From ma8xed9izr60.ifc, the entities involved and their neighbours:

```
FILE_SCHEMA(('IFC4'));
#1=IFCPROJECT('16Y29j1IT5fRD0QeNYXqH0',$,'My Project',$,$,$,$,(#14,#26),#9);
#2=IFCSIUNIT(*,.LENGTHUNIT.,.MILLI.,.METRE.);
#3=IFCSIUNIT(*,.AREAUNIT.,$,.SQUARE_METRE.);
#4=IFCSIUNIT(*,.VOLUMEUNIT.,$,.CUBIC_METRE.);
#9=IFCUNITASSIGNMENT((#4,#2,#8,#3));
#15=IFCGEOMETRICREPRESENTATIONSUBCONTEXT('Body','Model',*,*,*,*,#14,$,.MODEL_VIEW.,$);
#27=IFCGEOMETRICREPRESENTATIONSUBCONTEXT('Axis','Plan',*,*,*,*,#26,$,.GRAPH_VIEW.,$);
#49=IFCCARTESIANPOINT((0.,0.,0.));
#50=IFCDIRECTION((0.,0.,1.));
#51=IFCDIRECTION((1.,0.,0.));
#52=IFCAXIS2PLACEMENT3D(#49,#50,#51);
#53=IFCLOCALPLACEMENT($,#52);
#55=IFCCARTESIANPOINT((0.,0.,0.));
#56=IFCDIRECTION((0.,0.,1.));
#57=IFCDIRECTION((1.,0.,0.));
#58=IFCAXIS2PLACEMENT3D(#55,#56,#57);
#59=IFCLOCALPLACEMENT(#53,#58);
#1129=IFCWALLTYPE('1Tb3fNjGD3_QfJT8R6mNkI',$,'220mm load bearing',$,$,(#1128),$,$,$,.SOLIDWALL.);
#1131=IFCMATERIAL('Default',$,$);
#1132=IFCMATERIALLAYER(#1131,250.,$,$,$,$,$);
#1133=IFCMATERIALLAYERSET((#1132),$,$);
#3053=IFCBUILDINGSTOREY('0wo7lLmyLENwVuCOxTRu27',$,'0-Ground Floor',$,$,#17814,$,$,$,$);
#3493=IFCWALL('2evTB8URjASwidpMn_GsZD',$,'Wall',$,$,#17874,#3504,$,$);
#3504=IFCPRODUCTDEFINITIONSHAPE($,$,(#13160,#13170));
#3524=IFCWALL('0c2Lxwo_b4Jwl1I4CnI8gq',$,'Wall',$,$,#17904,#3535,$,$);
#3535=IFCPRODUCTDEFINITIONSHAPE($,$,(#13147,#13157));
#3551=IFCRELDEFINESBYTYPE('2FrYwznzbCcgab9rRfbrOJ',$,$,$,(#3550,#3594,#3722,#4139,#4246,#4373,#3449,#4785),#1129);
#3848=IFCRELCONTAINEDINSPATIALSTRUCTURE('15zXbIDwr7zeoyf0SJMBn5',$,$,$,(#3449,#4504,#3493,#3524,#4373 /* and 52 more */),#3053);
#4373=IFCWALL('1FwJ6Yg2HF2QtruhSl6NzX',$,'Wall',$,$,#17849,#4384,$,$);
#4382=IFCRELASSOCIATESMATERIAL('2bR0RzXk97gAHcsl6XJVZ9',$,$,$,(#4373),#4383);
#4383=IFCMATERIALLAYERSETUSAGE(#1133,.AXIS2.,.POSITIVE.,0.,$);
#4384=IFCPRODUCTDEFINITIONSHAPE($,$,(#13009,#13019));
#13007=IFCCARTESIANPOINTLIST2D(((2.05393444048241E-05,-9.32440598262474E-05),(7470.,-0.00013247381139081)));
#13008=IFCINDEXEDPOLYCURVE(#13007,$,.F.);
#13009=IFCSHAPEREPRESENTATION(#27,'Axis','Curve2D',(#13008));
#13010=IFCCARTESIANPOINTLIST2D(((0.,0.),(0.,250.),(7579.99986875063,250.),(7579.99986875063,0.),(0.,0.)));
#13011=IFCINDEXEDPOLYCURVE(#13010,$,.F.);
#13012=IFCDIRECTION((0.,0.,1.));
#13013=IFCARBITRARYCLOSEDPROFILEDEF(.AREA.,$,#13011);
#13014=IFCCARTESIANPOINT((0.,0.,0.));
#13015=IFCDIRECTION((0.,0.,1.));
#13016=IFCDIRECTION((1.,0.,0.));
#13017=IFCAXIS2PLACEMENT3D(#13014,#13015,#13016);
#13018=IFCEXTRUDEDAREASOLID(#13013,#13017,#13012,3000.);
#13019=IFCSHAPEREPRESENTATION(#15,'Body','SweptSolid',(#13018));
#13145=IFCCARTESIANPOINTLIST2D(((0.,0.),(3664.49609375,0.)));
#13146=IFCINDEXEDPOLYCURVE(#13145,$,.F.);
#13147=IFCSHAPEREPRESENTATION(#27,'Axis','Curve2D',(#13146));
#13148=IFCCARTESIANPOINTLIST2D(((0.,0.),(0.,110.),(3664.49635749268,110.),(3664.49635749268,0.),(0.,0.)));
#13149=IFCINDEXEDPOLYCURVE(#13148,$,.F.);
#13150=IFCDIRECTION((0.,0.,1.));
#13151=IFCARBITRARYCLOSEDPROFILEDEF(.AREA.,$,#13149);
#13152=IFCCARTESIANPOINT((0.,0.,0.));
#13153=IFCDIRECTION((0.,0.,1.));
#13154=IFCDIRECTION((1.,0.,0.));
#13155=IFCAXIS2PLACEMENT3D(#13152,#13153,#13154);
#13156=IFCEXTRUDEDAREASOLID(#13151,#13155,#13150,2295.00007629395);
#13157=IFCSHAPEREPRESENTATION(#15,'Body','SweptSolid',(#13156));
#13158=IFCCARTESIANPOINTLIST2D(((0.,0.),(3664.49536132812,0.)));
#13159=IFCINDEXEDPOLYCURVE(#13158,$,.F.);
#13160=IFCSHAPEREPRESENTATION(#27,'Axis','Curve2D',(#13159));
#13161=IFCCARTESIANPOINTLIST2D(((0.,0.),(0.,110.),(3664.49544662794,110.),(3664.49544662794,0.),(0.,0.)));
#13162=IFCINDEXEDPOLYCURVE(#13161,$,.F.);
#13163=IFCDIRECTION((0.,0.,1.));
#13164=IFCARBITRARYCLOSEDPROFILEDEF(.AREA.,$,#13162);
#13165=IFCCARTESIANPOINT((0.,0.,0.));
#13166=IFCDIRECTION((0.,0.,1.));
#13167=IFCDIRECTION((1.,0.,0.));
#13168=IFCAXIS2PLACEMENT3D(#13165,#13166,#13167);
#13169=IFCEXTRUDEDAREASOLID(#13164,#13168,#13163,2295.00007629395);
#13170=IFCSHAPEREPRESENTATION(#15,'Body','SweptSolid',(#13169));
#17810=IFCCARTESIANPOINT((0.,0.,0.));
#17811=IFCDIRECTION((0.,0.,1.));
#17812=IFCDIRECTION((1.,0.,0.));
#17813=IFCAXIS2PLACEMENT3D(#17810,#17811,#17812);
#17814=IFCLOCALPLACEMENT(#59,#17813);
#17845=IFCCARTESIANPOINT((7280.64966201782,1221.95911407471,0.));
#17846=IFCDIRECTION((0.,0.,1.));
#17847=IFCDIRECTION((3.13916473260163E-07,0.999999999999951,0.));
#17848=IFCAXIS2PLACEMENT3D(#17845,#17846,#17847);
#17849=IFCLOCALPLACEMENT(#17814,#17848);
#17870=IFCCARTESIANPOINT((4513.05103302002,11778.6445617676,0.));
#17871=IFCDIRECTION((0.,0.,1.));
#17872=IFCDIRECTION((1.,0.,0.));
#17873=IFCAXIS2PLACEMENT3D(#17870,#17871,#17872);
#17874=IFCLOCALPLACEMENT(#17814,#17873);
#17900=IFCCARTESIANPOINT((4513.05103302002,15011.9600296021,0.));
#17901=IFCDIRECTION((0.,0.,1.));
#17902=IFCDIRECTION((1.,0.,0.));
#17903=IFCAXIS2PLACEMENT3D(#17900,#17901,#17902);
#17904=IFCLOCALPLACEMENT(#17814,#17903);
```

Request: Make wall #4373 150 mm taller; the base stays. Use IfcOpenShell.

```python
import ifcopenshell
import ifcopenshell.geom
import ifcopenshell.util.representation
import ifcopenshell.util.shape
import ifcopenshell.util.unit

model = ifcopenshell.open("ma8xed9izr60.ifc")
unit_scale = ifcopenshell.util.unit.calculate_unit_scale(model)
settings = ifcopenshell.geom.settings()


def volume(element):
    """Net volume in cubic metres, openings subtracted."""
    shape = ifcopenshell.geom.create_shape(settings, element)
    return ifcopenshell.util.shape.get_volume(shape.geometry)


wall = model.by_guid("1FwJ6Yg2HF2QtruhSl6NzX")
before = volume(wall)

body = ifcopenshell.util.representation.get_representation(wall, "Model", "Body")
solid = body.Items[0]
old_height = solid.Depth
solid.Depth += 0.15 / unit_scale
after = volume(wall)

print(f"height {old_height:g} -> {solid.Depth:g}, volume {before:.3f} -> {after:.3f} m3")

model.write("ma8xed9izr60_updated.ifc")
```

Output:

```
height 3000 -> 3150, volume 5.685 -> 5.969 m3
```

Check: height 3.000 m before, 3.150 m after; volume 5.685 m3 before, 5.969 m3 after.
